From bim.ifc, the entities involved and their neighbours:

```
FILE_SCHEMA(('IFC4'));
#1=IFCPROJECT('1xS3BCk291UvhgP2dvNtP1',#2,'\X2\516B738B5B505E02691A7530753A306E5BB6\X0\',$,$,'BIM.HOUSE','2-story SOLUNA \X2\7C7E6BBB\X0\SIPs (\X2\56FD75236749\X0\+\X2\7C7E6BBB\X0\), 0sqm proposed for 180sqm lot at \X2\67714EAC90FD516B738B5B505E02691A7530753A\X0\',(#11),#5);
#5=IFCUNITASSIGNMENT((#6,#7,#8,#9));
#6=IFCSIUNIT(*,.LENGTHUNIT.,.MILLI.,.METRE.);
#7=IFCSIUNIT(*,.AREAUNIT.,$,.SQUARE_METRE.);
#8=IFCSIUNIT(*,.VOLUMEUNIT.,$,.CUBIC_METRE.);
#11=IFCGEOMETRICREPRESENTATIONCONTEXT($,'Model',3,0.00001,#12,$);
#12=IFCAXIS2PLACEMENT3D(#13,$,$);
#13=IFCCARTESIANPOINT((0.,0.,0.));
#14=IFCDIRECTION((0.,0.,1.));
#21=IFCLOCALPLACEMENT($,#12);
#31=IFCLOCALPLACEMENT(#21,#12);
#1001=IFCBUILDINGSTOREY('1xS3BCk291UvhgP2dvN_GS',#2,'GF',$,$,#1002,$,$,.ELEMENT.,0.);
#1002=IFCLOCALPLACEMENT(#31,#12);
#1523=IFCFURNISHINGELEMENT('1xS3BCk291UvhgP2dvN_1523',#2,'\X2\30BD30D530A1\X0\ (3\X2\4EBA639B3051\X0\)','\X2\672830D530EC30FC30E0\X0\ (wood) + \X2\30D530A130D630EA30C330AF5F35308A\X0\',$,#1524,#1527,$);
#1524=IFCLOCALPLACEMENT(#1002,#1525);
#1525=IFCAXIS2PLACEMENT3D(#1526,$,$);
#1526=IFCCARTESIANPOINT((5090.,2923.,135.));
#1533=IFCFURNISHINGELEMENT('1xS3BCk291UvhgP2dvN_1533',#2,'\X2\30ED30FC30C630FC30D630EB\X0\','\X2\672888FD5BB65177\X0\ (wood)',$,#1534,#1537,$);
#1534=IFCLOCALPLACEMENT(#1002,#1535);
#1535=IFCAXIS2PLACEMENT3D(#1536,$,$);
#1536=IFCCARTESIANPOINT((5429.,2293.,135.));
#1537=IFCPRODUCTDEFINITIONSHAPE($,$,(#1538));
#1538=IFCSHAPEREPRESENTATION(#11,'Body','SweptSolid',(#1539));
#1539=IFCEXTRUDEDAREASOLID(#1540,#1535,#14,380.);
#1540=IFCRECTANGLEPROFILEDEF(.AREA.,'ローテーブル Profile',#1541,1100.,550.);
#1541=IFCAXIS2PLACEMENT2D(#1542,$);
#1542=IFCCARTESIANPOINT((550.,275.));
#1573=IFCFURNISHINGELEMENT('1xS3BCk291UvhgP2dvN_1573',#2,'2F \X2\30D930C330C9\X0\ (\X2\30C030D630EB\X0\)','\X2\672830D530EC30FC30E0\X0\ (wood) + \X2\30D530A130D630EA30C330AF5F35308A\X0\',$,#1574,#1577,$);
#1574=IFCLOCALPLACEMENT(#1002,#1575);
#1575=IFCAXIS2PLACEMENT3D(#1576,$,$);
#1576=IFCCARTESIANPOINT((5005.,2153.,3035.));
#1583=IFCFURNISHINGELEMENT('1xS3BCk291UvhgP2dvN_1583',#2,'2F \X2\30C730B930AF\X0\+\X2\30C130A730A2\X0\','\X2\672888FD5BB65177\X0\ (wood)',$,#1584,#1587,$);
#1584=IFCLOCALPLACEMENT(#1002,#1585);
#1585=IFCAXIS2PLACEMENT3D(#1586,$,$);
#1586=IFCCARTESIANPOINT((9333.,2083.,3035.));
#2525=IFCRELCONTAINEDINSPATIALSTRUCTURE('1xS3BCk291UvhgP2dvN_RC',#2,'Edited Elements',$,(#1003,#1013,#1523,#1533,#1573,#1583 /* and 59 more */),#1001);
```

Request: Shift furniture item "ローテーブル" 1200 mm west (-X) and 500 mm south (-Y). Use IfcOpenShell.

```python
import ifcopenshell
import ifcopenshell.api.geometry
import ifcopenshell.util.placement

model = ifcopenshell.open("bim.ifc")

item = model.by_guid("1xS3BCk291UvhgP2dvN_1533")
matrix = ifcopenshell.util.placement.get_local_placement(item.ObjectPlacement)
matrix[0, 3] -= 1200.0
matrix[1, 3] -= 500.0
ifcopenshell.api.geometry.edit_object_placement(model, product=item, matrix=matrix, is_si=False)

print(ifcopenshell.util.placement.get_local_placement(item.ObjectPlacement).round(3) + 0.0)

model.write("bim_edited.ifc")
```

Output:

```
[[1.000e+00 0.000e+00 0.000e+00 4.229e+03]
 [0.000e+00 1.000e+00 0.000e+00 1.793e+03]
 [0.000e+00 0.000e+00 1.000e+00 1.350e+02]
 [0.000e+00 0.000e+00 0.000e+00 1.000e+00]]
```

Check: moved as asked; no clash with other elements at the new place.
